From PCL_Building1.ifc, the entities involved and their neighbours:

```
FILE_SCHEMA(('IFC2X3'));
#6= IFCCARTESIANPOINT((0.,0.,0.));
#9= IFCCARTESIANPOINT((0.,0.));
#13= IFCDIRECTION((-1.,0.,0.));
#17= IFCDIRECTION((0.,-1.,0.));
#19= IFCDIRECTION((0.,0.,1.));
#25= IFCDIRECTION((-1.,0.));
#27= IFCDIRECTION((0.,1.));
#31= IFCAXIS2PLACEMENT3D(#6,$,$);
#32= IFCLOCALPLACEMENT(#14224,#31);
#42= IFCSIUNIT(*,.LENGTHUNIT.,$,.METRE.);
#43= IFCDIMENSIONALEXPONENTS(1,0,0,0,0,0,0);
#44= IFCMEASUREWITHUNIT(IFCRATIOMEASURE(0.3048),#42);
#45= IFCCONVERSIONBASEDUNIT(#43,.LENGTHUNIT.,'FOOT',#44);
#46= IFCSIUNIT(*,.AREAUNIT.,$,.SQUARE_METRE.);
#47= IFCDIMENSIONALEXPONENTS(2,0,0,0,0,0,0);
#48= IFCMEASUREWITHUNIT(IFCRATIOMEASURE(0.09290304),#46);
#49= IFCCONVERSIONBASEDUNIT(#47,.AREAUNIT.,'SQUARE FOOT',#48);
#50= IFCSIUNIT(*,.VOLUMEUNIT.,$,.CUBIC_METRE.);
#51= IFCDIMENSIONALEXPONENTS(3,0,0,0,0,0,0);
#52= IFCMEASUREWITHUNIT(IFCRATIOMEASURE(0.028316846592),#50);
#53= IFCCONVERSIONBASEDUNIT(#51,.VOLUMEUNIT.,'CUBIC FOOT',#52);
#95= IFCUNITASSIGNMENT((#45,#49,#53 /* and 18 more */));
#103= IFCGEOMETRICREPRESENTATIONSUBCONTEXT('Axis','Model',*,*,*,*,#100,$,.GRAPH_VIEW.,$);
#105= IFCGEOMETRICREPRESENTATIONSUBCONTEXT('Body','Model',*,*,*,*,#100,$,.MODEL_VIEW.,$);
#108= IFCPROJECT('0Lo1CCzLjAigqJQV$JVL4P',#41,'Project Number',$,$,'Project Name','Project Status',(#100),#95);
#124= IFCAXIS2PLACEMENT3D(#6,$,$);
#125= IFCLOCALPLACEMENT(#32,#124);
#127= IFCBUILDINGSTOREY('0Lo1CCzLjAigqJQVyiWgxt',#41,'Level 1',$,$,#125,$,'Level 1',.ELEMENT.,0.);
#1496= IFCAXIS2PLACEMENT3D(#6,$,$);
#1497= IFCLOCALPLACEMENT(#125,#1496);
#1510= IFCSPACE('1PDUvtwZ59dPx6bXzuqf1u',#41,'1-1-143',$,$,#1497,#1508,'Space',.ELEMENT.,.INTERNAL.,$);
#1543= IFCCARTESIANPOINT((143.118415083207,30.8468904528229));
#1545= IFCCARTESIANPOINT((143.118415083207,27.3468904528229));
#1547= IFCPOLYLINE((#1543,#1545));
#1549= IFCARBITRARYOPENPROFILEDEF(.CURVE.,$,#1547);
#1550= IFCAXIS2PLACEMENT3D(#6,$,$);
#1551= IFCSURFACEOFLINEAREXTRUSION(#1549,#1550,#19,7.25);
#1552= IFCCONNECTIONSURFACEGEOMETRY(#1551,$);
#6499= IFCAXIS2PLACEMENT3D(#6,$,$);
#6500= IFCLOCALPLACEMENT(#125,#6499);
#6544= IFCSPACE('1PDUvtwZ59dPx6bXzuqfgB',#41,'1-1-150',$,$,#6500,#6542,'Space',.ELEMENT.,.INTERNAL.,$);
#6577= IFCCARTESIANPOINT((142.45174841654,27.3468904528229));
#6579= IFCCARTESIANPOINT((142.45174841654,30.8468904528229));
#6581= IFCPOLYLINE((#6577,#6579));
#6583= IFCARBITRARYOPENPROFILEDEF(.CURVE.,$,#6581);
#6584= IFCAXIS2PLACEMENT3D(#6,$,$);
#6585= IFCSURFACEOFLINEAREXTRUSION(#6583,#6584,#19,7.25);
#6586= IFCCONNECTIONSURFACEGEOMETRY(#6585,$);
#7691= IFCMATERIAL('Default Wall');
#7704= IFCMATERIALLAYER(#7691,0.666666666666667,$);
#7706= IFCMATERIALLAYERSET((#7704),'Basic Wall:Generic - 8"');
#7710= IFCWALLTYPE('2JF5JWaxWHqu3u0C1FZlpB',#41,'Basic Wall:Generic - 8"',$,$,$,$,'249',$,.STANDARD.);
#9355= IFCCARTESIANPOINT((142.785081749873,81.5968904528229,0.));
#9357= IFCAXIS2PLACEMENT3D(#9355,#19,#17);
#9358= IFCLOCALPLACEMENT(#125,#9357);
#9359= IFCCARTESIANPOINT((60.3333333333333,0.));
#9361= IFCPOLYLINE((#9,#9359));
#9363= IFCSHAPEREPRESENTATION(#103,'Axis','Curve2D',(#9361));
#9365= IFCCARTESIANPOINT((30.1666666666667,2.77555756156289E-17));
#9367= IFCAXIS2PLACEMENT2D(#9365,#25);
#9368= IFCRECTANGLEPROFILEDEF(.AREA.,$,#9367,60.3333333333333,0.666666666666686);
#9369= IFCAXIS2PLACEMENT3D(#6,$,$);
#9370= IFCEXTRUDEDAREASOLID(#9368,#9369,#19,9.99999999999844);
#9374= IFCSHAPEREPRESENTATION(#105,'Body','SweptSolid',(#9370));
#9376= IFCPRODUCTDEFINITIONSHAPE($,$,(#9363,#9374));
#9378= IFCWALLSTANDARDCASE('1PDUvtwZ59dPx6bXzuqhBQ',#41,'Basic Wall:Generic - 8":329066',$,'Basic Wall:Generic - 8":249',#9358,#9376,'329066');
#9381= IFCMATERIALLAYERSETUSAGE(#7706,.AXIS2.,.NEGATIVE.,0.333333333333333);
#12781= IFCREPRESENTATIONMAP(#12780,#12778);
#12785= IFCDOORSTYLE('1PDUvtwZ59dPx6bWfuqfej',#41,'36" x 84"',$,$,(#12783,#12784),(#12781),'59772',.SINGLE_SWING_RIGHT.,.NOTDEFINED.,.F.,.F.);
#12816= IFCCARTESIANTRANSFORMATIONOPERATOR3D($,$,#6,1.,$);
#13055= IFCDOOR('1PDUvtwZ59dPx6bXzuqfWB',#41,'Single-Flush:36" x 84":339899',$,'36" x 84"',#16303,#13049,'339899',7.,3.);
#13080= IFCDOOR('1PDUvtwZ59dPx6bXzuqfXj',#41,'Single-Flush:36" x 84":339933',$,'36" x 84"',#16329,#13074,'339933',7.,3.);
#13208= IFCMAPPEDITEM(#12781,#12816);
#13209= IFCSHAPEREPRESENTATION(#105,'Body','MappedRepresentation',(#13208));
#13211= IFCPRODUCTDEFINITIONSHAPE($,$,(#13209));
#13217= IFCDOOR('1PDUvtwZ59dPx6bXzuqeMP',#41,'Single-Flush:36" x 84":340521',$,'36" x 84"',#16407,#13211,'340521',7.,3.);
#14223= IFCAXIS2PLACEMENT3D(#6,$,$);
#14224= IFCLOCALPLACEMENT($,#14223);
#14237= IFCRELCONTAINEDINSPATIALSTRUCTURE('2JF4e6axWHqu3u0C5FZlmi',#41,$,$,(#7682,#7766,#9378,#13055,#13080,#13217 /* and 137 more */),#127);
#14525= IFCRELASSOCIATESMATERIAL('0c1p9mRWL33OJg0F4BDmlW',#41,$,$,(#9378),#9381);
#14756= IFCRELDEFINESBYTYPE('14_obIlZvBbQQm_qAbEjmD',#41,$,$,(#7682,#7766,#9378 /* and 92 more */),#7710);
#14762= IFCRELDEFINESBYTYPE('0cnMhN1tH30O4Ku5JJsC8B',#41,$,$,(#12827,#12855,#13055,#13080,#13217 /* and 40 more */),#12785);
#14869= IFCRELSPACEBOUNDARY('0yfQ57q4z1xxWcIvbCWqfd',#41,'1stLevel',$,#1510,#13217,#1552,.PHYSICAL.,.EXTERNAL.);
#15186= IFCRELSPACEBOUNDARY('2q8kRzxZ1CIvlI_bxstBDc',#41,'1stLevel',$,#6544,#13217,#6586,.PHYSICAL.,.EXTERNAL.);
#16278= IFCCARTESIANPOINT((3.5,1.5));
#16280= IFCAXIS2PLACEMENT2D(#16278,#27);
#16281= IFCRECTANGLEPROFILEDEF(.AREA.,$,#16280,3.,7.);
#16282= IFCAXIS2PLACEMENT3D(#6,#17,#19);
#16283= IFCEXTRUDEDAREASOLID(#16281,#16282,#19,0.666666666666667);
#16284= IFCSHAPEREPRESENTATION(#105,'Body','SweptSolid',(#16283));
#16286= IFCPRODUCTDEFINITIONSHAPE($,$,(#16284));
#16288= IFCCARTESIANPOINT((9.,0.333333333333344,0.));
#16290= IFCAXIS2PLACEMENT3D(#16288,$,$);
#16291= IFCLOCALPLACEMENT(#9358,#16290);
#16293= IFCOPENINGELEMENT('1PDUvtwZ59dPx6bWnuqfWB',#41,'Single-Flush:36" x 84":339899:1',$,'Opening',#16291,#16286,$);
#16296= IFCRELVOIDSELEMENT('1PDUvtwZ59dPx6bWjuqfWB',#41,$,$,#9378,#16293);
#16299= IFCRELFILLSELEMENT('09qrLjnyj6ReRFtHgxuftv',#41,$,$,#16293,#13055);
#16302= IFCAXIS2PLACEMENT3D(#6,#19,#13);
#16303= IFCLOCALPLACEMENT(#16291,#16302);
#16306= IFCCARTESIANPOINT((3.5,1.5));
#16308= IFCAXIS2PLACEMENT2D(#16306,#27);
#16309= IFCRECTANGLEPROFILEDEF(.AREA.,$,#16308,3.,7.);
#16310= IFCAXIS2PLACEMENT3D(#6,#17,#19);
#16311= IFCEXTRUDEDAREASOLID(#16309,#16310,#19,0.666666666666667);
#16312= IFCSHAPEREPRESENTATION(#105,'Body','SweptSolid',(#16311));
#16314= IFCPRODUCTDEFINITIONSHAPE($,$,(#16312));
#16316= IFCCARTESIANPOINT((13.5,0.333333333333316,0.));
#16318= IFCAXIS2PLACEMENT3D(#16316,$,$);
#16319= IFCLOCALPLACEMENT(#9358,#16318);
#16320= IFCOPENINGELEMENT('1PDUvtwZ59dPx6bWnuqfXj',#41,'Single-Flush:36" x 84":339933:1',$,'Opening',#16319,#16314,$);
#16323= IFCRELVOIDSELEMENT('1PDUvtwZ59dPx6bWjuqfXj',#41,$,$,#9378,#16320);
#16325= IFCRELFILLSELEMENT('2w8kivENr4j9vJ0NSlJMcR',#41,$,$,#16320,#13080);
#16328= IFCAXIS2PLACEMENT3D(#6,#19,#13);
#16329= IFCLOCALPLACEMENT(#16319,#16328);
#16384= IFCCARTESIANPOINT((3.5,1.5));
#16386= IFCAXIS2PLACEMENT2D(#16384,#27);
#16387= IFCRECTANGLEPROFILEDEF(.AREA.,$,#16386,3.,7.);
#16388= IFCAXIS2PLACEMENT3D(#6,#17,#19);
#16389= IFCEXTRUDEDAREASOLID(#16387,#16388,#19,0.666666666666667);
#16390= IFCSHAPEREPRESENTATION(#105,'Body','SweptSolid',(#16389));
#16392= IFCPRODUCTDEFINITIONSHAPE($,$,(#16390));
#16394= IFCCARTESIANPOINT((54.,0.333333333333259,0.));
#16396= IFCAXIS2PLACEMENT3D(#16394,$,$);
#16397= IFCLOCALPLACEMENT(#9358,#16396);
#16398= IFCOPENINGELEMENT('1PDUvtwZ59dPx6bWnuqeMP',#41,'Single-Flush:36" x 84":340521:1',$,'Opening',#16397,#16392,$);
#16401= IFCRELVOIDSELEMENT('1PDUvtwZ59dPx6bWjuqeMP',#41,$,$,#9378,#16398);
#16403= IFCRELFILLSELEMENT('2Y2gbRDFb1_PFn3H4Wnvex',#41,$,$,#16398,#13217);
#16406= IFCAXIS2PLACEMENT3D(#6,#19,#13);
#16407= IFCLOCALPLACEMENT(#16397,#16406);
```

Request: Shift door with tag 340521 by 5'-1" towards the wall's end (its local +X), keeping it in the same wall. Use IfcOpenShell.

```python
import numpy as np
import ifcopenshell
import ifcopenshell.api.geometry
import ifcopenshell.util.placement
import ifcopenshell.util.unit

model = ifcopenshell.open("PCL_Building1.ifc")
unit_scale = ifcopenshell.util.unit.calculate_unit_scale(model)

door = model.by_guid("1PDUvtwZ59dPx6bXzuqeMP")
opening = door.FillsVoids[0].RelatingOpeningElement
wall = opening.VoidsElements[0].RelatingBuildingElement

wall_matrix = ifcopenshell.util.placement.get_local_placement(wall.ObjectPlacement)
shift = wall_matrix[:3, 0] * 61 * 0.0254 / unit_scale
before = ifcopenshell.util.placement.get_local_placement(door.ObjectPlacement)[:3, 3].copy()

# The door is placed relative to its opening, so it follows when the opening moves.
matrix = ifcopenshell.util.placement.get_local_placement(opening.ObjectPlacement)
matrix[:3, 3] += shift
ifcopenshell.api.geometry.edit_object_placement(
    model, product=opening, matrix=matrix, is_si=False, should_transform_children=True
)

# Space boundary surfaces are stored in each space's coordinates; move them too.
for rel in door.ProvidesBoundaries:
    if not rel.ConnectionGeometry:
        continue
    surface = rel.ConnectionGeometry.SurfaceOnRelatingElement
    space_matrix = ifcopenshell.util.placement.get_local_placement(rel.RelatingSpace.ObjectPlacement)
    point = np.array(surface.Position.Location.Coordinates) + space_matrix[:3, :3].T @ shift
    surface.Position = model.createIfcAxis2Placement3D(
        model.createIfcCartesianPoint(point.tolist()), surface.Position.Axis, surface.Position.RefDirection
    )

after = ifcopenshell.util.placement.get_local_placement(door.ObjectPlacement)[:3, 3]
print("door moved by", (after - before).round(3) + 0.0)

model.write("PCL_Building1_rev.ifc")
```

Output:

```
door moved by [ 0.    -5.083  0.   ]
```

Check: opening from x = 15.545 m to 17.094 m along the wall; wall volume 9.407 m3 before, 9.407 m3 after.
